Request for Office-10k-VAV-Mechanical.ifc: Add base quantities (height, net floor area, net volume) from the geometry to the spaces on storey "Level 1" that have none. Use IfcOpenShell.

First a look at what the model holds.

```python
import ifcopenshell
import ifcopenshell.util.element
import ifcopenshell.util.unit

model = ifcopenshell.open("Office-10k-VAV-Mechanical.ifc")
print(model.schema)
for unit_type in ("LENGTHUNIT", "AREAUNIT", "VOLUMEUNIT"):
    print(unit_type, ifcopenshell.util.unit.calculate_unit_scale(model, unit_type))
storey = next(s for s in model.by_type("IfcBuildingStorey") if s.Name == "Level 1")
spaces = [e for e in ifcopenshell.util.element.get_decomposition(storey) if e.is_a("IfcSpace")]
for e in sorted(spaces, key=lambda e: e.id()):
    print(e.id(), e.is_a(), e.Name, list(ifcopenshell.util.element.get_psets(e, qtos_only=True)), sep=" | ")
```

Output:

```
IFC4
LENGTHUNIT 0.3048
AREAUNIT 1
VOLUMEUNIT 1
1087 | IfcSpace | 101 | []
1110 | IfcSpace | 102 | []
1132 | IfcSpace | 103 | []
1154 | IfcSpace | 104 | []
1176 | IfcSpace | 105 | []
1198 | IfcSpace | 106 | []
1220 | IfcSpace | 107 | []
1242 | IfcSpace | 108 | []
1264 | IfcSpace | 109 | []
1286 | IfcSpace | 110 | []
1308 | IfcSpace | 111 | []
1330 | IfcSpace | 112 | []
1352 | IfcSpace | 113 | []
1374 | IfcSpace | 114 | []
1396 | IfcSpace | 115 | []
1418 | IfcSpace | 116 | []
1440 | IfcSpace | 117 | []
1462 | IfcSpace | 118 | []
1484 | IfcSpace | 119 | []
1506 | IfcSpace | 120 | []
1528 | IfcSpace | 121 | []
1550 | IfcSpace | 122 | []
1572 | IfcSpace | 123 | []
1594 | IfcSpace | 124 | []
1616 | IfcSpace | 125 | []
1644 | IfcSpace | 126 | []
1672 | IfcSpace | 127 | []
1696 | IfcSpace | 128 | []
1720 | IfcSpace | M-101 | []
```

```python
import ifcopenshell
import ifcopenshell.api.pset
import ifcopenshell.geom
import ifcopenshell.util.element
import ifcopenshell.util.shape
import ifcopenshell.util.unit

model = ifcopenshell.open("Office-10k-VAV-Mechanical.ifc")
unit_scale = ifcopenshell.util.unit.calculate_unit_scale(model)
area_scale = ifcopenshell.util.unit.calculate_unit_scale(model, "AREAUNIT")
volume_scale = ifcopenshell.util.unit.calculate_unit_scale(model, "VOLUMEUNIT")
settings = ifcopenshell.geom.settings()

storey = next(s for s in model.by_type("IfcBuildingStorey") if s.Name == "Level 1")
spaces = [e for e in ifcopenshell.util.element.get_decomposition(storey) if e.is_a("IfcSpace")]

for e in sorted(spaces, key=lambda e: e.id()):
    if ifcopenshell.util.element.get_psets(e, qtos_only=True, should_inherit=False):
        continue
    # Geometry comes back in metres, in the element's own axes.
    shape = ifcopenshell.geom.create_shape(settings, e)
    values = {
        "Height": ifcopenshell.util.shape.get_z(shape.geometry) / unit_scale,
        "NetFloorArea": ifcopenshell.util.shape.get_footprint_area(shape.geometry) / area_scale,
        "NetVolume": ifcopenshell.util.shape.get_volume(shape.geometry) / volume_scale,
    }
    qto = ifcopenshell.api.pset.add_qto(model, product=e, name="Qto_SpaceBaseQuantities")
    ifcopenshell.api.pset.edit_qto(model, qto=qto, properties=values)
    print(e.id(), {k: round(v, 3) for k, v in values.items()})

model.write("Office-10k-VAV-Mechanical_v2.ifc")
```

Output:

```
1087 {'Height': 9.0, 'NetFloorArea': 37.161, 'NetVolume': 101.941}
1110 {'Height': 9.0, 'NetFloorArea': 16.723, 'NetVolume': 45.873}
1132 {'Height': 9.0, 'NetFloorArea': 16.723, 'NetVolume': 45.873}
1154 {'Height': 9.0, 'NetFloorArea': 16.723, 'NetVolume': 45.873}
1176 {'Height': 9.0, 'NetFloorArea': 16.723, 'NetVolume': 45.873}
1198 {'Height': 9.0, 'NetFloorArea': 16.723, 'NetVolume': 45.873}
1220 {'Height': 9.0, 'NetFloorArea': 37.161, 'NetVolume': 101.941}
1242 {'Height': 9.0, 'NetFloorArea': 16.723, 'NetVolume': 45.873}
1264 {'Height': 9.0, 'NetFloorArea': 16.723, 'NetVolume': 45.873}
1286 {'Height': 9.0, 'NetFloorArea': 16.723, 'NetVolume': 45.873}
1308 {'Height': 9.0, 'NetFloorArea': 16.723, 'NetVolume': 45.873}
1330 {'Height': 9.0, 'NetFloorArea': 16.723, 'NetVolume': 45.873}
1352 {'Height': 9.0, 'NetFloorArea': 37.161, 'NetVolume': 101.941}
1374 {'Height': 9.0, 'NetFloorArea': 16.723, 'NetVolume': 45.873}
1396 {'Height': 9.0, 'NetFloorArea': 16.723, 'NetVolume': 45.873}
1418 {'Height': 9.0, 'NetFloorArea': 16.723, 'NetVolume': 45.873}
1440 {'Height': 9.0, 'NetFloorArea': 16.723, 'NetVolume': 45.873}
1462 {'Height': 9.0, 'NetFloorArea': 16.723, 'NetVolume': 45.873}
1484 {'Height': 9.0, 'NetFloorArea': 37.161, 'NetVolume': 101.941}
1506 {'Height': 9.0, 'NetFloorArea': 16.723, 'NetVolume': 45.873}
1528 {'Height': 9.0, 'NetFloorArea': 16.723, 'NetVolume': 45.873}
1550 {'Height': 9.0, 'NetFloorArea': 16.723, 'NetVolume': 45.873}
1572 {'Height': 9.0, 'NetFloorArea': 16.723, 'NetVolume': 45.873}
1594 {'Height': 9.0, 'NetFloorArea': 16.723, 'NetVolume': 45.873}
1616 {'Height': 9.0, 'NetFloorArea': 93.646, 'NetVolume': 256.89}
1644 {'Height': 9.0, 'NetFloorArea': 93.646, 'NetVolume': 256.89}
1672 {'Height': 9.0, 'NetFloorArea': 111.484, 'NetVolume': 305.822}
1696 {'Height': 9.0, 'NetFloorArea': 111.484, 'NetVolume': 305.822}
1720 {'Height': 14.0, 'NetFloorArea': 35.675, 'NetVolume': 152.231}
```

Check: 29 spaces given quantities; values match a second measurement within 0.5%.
